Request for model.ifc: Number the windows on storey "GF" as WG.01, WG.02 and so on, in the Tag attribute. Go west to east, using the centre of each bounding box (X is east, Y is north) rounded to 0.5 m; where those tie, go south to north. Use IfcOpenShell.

First a look at what the model holds.

```python
import ifcopenshell
import ifcopenshell.util.element
import ifcopenshell.util.placement

model = ifcopenshell.open("model.ifc")
print(model.schema)
storey = next(s for s in model.by_type("IfcBuildingStorey") if s.Name == "GF")
windows = [e for e in ifcopenshell.util.element.get_decomposition(storey) if e.is_a("IfcWindow")]
for e in sorted(windows, key=lambda e: e.id()):
    origin = ifcopenshell.util.placement.get_local_placement(e.ObjectPlacement)[:3, 3]
    print(e.id(), e.Tag, e.Name, origin.round(2) + 0.0, sep=" | ")
```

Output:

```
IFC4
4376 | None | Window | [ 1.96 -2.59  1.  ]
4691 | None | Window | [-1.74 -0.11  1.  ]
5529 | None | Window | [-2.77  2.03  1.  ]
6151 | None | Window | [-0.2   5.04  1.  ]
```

```python
import ifcopenshell
import ifcopenshell.geom
import ifcopenshell.util.element
import ifcopenshell.util.shape

model = ifcopenshell.open("model.ifc")
settings = ifcopenshell.geom.settings()
settings.set("use-world-coords", True)


def centre(element):
    shape = ifcopenshell.geom.create_shape(settings, element)
    return ifcopenshell.util.shape.get_bbox_centroid(shape.geometry)


storey = next(s for s in model.by_type("IfcBuildingStorey") if s.Name == "GF")
windows = [e for e in ifcopenshell.util.element.get_decomposition(storey) if e.is_a("IfcWindow")]

# Insertion points can sit at a corner or the storey origin, so sort by the geometry (in metres).
centres = {e: centre(e) for e in windows}
windows.sort(key=lambda e: (round(centres[e][0] / 0.5), centres[e][1]))

for i, e in enumerate(windows, start=1):
    number = f"WG.{i:02d}"
    e.Tag = number
    print(e.id(), number)

model.write("model_v2.ifc")
```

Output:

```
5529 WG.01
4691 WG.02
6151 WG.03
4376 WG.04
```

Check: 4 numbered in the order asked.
